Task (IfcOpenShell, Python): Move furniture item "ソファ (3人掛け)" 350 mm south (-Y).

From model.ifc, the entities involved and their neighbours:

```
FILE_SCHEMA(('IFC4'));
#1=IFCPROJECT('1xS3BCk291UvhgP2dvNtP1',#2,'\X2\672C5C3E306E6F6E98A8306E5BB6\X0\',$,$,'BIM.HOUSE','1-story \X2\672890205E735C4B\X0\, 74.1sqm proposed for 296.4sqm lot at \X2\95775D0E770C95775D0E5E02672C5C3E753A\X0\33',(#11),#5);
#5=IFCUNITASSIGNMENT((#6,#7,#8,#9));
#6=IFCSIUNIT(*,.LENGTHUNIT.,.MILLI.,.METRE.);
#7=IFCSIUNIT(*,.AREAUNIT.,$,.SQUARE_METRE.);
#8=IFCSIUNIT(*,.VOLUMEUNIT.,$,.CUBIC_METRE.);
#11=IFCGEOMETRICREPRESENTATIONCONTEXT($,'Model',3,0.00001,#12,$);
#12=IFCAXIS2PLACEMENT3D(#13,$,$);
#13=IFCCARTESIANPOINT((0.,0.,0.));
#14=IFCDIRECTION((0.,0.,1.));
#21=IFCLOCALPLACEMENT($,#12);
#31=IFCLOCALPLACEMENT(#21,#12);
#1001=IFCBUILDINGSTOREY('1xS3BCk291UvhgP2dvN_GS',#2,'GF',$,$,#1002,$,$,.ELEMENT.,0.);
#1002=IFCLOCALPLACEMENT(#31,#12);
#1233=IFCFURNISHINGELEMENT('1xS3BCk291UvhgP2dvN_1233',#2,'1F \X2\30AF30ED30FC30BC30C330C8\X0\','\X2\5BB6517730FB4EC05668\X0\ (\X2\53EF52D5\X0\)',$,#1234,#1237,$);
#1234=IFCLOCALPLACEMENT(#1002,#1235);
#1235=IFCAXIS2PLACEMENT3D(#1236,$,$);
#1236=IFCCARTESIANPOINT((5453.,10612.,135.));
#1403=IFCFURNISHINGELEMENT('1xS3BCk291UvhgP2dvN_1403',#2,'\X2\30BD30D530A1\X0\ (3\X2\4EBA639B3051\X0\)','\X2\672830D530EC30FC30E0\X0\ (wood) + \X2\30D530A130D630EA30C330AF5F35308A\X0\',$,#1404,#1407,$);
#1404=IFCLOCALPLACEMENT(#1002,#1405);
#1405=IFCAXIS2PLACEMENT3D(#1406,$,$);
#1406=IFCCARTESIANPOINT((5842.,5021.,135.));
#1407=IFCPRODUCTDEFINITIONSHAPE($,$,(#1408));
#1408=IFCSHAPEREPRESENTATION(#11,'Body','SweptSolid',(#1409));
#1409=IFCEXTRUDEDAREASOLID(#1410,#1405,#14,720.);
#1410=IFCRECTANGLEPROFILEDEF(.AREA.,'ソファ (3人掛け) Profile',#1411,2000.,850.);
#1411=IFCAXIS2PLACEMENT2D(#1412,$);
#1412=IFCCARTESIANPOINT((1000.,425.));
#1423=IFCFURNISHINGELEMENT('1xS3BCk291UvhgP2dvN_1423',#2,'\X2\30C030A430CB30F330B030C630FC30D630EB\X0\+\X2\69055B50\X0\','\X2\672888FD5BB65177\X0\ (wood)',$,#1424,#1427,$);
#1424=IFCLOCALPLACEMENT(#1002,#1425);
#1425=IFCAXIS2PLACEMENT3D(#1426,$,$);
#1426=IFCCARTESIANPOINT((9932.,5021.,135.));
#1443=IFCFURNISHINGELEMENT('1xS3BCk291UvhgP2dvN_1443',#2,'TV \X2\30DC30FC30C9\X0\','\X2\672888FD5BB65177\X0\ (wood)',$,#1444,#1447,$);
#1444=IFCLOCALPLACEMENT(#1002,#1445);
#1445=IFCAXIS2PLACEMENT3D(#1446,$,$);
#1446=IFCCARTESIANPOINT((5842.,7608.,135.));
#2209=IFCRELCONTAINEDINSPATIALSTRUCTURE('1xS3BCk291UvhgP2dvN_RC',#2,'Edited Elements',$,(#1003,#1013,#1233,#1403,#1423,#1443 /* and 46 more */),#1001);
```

```python
import ifcopenshell
import ifcopenshell.api.geometry
import ifcopenshell.util.placement
import ifcopenshell.util.unit

model = ifcopenshell.open("model.ifc")
unit_scale = ifcopenshell.util.unit.calculate_unit_scale(model)

item = model.by_guid("1xS3BCk291UvhgP2dvN_1403")
matrix = ifcopenshell.util.placement.get_local_placement(item.ObjectPlacement)
matrix[1, 3] -= 0.35 / unit_scale
ifcopenshell.api.geometry.edit_object_placement(model, product=item, matrix=matrix, is_si=False)

print(ifcopenshell.util.placement.get_local_placement(item.ObjectPlacement).round(3) + 0.0)

model.write("model_v2.ifc")
```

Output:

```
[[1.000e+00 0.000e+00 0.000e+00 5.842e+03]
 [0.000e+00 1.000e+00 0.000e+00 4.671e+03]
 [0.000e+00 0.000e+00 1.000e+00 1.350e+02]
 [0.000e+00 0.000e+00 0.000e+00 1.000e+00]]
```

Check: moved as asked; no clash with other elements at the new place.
